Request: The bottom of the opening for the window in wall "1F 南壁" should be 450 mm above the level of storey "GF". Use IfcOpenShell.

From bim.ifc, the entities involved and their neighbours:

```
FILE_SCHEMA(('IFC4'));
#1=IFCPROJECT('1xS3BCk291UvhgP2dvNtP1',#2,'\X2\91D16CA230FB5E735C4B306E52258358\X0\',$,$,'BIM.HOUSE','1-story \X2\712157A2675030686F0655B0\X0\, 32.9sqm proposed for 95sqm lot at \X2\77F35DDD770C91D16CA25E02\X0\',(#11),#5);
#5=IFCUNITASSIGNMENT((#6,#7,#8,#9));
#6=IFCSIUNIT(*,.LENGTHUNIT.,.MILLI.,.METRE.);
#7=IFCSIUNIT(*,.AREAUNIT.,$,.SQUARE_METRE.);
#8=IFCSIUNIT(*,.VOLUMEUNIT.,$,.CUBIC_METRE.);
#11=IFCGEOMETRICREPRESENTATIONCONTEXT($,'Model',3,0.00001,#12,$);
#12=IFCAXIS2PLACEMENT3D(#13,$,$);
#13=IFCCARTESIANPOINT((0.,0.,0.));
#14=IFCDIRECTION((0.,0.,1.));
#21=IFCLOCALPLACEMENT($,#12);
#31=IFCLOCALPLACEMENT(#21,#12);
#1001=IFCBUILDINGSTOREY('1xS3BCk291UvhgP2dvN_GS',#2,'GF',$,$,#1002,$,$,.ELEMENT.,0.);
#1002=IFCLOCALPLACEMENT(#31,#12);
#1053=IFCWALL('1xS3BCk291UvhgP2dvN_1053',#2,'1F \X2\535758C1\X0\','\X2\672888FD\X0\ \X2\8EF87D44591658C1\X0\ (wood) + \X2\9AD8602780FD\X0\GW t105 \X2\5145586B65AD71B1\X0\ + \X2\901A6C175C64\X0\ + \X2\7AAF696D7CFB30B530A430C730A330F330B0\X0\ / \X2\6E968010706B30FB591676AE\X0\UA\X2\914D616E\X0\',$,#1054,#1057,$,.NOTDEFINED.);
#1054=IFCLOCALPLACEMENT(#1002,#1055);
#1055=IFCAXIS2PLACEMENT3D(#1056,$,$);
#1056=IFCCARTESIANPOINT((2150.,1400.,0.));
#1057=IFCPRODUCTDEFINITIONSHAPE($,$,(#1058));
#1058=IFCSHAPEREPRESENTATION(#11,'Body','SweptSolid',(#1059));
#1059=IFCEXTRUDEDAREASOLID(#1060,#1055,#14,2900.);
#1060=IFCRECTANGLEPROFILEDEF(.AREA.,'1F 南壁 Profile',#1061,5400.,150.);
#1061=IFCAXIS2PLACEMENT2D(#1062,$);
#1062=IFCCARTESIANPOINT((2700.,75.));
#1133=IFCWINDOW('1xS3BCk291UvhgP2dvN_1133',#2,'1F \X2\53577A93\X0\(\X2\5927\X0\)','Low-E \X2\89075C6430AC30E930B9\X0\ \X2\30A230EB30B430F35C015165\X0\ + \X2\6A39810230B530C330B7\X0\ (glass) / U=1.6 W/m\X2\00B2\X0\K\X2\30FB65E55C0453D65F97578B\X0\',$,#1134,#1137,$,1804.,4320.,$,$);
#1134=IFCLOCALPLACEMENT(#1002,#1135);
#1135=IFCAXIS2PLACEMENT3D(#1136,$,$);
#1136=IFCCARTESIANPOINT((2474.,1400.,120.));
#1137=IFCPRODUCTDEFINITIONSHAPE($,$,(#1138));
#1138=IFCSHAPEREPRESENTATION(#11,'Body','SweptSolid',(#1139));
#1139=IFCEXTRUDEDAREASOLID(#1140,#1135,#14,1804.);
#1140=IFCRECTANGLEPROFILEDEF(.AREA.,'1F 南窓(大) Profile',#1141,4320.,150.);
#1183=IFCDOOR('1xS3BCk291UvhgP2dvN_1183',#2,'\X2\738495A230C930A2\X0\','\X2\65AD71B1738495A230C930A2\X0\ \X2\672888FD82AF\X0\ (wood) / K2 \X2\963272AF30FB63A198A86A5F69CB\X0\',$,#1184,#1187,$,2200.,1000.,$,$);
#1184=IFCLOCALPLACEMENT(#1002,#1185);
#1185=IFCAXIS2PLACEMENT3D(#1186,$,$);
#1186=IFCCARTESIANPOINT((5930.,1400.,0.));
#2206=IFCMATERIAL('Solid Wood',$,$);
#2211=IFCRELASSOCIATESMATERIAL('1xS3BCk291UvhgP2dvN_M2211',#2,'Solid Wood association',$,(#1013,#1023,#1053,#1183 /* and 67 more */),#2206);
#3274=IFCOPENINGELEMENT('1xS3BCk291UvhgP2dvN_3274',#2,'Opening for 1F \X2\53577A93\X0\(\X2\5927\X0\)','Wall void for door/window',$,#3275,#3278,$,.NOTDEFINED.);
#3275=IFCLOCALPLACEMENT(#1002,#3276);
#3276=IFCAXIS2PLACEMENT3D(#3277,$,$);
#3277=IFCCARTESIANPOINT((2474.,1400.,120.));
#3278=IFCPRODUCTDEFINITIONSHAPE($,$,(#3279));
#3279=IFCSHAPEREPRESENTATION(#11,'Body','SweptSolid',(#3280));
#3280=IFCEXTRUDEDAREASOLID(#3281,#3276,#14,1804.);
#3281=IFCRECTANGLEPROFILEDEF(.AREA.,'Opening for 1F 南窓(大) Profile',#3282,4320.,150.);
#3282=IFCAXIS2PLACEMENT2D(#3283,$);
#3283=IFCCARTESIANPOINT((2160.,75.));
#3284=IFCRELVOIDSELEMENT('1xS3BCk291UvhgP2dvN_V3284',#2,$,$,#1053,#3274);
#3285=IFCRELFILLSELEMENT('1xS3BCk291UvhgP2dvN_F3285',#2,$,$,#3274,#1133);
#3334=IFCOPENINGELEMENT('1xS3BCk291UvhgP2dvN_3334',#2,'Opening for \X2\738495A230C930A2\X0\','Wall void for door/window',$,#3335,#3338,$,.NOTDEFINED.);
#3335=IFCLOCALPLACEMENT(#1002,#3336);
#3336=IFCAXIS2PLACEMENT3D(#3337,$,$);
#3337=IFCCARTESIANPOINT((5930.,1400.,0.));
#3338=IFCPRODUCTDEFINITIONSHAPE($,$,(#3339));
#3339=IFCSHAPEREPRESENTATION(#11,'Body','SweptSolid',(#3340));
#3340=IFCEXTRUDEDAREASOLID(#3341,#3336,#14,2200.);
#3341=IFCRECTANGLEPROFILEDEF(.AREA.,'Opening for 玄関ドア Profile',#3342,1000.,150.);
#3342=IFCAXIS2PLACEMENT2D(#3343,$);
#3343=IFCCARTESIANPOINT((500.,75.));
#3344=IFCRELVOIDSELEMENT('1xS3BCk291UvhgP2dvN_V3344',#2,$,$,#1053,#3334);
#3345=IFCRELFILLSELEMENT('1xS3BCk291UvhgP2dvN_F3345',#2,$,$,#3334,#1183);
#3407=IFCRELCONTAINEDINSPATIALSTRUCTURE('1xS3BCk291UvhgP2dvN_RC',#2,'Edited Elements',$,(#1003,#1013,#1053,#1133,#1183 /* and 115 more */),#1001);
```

```python
import numpy as np
import ifcopenshell
import ifcopenshell.api.geometry
import ifcopenshell.geom
import ifcopenshell.util.element
import ifcopenshell.util.placement
import ifcopenshell.util.shape
import ifcopenshell.util.unit

model = ifcopenshell.open("bim.ifc")
unit_scale = ifcopenshell.util.unit.calculate_unit_scale(model)

window = model.by_guid("1xS3BCk291UvhgP2dvN_1133")
opening = window.FillsVoids[0].RelatingOpeningElement
storey = ifcopenshell.util.element.get_container(window, ifc_class="IfcBuildingStorey")
level = ifcopenshell.util.placement.get_local_placement(storey.ObjectPlacement)[2, 3]

# The opening's origin need not be at the sill, so measure its lowest point.
shape = ifcopenshell.geom.create_shape(ifcopenshell.geom.settings(), opening)
bottom = ifcopenshell.util.shape.get_shape_bottom_elevation(shape, shape.geometry) / unit_scale
dz = level + 0.45 / unit_scale - bottom

shift = np.array([0.0, 0.0, dz])
# The window is not placed relative to its opening, so move both.
for product in (opening, window):
    matrix = ifcopenshell.util.placement.get_local_placement(product.ObjectPlacement)
    matrix[:3, 3] += shift
    ifcopenshell.api.geometry.edit_object_placement(model, product=product, matrix=matrix, is_si=False)

print(f"moved by {dz * unit_scale:+.3f} m")

model.write("bim-out.ifc")
```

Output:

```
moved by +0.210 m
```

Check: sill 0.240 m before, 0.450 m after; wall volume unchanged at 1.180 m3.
